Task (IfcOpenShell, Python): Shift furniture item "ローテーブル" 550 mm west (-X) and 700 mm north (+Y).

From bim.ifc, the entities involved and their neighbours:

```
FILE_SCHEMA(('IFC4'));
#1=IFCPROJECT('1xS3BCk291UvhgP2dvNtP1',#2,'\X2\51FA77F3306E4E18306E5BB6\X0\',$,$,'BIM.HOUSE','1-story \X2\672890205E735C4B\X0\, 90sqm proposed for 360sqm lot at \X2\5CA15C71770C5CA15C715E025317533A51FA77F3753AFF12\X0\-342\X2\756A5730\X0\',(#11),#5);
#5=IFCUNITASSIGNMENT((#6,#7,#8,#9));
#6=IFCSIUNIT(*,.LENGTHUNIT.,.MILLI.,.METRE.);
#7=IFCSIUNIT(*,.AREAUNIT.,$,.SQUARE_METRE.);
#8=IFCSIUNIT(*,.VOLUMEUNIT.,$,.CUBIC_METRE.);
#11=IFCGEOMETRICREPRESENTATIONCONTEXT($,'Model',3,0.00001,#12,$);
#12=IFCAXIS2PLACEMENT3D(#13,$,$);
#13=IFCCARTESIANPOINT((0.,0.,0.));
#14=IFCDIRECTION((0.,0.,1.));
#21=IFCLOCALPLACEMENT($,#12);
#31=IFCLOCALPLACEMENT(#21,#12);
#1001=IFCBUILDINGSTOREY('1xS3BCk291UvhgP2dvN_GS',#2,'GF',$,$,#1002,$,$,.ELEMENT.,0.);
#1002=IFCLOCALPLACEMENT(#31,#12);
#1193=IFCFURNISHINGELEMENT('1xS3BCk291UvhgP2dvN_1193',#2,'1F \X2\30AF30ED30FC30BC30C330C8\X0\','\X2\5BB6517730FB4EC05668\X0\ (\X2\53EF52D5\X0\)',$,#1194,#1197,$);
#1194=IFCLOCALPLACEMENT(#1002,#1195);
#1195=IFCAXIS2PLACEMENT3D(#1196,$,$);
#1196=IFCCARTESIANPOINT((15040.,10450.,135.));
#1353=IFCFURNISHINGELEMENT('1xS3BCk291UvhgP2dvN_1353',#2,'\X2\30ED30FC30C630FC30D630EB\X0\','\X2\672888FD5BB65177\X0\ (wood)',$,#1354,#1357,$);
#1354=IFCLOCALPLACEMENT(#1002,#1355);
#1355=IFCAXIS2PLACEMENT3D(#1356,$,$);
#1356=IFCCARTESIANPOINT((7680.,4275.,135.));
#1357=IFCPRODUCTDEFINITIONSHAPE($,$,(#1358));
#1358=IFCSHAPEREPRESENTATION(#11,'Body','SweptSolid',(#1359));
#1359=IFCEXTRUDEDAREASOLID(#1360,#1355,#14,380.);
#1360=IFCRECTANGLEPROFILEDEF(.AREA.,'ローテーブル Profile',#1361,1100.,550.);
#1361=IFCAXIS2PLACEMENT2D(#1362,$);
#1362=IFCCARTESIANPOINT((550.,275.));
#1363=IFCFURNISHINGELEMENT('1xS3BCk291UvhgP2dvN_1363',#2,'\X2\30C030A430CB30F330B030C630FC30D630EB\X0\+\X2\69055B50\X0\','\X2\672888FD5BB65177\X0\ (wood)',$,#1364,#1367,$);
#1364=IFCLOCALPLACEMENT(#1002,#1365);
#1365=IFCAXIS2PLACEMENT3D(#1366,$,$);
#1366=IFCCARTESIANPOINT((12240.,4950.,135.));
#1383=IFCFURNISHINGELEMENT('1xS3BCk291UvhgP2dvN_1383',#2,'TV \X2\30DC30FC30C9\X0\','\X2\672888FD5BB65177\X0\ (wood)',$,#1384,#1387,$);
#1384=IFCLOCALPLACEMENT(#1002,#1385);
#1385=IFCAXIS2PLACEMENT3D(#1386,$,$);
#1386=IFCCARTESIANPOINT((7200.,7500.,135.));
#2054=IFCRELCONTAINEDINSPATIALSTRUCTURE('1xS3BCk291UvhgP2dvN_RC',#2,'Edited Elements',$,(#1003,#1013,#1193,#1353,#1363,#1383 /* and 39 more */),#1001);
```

```python
import ifcopenshell
import ifcopenshell.api.geometry
import ifcopenshell.util.placement
import ifcopenshell.util.unit

model = ifcopenshell.open("bim.ifc")
unit_scale = ifcopenshell.util.unit.calculate_unit_scale(model)

item = model.by_guid("1xS3BCk291UvhgP2dvN_1353")
matrix = ifcopenshell.util.placement.get_local_placement(item.ObjectPlacement)
matrix[0, 3] -= 0.55 / unit_scale
matrix[1, 3] += 0.7 / unit_scale
ifcopenshell.api.geometry.edit_object_placement(model, product=item, matrix=matrix, is_si=False)

print(ifcopenshell.util.placement.get_local_placement(item.ObjectPlacement).round(3) + 0.0)

model.write("bim-out.ifc")
```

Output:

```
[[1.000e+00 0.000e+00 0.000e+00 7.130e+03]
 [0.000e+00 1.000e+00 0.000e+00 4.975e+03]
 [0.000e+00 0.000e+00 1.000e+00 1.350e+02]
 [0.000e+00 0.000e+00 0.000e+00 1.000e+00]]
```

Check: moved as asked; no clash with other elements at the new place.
